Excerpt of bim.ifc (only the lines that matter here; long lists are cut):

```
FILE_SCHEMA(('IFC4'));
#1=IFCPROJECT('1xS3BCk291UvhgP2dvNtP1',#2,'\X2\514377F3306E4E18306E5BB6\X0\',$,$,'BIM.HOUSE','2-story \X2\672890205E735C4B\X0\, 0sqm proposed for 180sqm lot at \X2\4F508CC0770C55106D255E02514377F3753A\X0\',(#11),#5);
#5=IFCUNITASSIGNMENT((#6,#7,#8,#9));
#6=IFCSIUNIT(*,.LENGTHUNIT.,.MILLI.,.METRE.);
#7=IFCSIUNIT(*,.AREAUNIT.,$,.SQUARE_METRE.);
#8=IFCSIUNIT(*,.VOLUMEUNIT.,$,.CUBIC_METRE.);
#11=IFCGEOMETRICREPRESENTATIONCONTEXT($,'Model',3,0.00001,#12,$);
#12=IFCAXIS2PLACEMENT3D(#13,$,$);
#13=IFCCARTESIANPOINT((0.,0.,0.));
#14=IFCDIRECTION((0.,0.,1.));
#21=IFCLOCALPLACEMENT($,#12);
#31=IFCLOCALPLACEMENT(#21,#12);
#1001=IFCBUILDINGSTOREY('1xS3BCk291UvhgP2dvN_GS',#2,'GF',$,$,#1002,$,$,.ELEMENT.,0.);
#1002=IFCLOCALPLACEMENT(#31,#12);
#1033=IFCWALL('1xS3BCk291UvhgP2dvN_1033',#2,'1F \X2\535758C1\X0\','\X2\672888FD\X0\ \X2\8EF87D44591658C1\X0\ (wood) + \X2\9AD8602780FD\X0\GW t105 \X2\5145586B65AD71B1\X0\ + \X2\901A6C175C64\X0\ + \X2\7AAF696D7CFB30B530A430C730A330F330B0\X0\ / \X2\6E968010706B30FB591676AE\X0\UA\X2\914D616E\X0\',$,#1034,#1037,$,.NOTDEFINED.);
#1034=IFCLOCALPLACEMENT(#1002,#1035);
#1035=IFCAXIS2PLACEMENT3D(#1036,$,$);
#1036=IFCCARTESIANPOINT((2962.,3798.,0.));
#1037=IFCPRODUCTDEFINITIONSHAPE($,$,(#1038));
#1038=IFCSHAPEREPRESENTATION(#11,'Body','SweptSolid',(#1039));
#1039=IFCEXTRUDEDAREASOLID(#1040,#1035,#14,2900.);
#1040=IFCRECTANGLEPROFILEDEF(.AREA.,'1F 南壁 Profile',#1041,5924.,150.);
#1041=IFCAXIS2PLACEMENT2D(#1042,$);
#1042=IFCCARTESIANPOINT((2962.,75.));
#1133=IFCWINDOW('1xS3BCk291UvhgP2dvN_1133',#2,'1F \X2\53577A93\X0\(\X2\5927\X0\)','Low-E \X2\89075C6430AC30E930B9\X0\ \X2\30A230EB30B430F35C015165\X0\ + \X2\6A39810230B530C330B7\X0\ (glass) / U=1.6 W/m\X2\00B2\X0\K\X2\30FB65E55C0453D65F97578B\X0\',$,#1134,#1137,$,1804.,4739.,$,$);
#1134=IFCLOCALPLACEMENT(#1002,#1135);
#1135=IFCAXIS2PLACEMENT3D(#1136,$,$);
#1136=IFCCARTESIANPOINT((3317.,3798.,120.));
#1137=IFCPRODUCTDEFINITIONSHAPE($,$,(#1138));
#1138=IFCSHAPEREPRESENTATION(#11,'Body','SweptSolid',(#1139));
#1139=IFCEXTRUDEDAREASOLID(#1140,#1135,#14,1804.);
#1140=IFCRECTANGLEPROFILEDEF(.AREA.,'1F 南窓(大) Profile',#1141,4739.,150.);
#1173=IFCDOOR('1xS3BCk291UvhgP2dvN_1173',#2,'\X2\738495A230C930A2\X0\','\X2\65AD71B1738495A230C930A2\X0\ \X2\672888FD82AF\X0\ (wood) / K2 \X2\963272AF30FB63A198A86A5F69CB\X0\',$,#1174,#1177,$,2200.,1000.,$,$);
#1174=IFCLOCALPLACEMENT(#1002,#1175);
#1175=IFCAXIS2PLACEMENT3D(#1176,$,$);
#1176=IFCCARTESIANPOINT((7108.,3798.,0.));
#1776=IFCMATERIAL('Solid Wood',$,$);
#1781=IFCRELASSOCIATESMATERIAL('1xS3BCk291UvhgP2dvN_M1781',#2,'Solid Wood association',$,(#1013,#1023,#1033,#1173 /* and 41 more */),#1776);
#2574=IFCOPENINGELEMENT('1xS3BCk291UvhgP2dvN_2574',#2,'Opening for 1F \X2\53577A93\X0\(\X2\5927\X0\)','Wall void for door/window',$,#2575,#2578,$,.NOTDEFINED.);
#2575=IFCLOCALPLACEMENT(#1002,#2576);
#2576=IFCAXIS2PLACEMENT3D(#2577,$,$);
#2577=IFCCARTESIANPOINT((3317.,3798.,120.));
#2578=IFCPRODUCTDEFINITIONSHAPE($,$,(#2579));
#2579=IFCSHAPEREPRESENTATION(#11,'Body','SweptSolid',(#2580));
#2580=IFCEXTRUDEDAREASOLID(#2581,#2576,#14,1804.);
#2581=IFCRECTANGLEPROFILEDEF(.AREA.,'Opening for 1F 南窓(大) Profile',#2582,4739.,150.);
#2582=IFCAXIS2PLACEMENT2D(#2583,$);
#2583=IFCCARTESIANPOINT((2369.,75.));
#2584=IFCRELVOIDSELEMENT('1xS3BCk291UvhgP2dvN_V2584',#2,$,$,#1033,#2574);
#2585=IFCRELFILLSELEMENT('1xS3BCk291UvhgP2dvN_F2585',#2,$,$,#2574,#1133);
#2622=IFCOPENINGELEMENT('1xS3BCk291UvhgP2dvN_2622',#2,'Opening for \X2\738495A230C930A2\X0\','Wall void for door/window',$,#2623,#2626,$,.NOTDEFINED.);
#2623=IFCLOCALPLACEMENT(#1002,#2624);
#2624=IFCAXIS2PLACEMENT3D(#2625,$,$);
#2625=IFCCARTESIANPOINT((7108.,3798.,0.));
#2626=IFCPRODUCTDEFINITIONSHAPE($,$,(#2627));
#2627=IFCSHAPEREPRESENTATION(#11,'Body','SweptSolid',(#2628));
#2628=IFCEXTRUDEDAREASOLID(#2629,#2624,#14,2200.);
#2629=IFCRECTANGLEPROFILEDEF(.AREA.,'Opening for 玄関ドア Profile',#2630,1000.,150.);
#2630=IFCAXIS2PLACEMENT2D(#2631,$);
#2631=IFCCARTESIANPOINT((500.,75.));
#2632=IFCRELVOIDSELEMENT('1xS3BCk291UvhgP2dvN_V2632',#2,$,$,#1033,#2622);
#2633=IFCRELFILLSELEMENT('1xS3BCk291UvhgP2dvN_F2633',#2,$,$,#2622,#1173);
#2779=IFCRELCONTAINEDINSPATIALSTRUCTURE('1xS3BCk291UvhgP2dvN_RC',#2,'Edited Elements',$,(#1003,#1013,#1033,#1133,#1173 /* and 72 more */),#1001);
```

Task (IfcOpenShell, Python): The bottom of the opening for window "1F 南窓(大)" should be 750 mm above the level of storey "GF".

```python
import numpy as np
import ifcopenshell
import ifcopenshell.api.geometry
import ifcopenshell.geom
import ifcopenshell.util.element
import ifcopenshell.util.placement
import ifcopenshell.util.shape
import ifcopenshell.util.unit

model = ifcopenshell.open("bim.ifc")
unit_scale = ifcopenshell.util.unit.calculate_unit_scale(model)

window = model.by_guid("1xS3BCk291UvhgP2dvN_1133")
opening = window.FillsVoids[0].RelatingOpeningElement
storey = ifcopenshell.util.element.get_container(window, ifc_class="IfcBuildingStorey")
level = ifcopenshell.util.placement.get_local_placement(storey.ObjectPlacement)[2, 3]

# The opening's origin need not be at the sill, so measure its lowest point.
shape = ifcopenshell.geom.create_shape(ifcopenshell.geom.settings(), opening)
bottom = ifcopenshell.util.shape.get_shape_bottom_elevation(shape, shape.geometry) / unit_scale
dz = level + 0.75 / unit_scale - bottom

shift = np.array([0.0, 0.0, dz])
# The window is not placed relative to its opening, so move both.
for product in (opening, window):
    matrix = ifcopenshell.util.placement.get_local_placement(product.ObjectPlacement)
    matrix[:3, 3] += shift
    ifcopenshell.api.geometry.edit_object_placement(model, product=product, matrix=matrix, is_si=False)

print(f"moved by {dz * unit_scale:+.3f} m")

model.write("bim_updated.ifc")
```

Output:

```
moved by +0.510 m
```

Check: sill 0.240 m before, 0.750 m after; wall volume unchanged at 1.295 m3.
